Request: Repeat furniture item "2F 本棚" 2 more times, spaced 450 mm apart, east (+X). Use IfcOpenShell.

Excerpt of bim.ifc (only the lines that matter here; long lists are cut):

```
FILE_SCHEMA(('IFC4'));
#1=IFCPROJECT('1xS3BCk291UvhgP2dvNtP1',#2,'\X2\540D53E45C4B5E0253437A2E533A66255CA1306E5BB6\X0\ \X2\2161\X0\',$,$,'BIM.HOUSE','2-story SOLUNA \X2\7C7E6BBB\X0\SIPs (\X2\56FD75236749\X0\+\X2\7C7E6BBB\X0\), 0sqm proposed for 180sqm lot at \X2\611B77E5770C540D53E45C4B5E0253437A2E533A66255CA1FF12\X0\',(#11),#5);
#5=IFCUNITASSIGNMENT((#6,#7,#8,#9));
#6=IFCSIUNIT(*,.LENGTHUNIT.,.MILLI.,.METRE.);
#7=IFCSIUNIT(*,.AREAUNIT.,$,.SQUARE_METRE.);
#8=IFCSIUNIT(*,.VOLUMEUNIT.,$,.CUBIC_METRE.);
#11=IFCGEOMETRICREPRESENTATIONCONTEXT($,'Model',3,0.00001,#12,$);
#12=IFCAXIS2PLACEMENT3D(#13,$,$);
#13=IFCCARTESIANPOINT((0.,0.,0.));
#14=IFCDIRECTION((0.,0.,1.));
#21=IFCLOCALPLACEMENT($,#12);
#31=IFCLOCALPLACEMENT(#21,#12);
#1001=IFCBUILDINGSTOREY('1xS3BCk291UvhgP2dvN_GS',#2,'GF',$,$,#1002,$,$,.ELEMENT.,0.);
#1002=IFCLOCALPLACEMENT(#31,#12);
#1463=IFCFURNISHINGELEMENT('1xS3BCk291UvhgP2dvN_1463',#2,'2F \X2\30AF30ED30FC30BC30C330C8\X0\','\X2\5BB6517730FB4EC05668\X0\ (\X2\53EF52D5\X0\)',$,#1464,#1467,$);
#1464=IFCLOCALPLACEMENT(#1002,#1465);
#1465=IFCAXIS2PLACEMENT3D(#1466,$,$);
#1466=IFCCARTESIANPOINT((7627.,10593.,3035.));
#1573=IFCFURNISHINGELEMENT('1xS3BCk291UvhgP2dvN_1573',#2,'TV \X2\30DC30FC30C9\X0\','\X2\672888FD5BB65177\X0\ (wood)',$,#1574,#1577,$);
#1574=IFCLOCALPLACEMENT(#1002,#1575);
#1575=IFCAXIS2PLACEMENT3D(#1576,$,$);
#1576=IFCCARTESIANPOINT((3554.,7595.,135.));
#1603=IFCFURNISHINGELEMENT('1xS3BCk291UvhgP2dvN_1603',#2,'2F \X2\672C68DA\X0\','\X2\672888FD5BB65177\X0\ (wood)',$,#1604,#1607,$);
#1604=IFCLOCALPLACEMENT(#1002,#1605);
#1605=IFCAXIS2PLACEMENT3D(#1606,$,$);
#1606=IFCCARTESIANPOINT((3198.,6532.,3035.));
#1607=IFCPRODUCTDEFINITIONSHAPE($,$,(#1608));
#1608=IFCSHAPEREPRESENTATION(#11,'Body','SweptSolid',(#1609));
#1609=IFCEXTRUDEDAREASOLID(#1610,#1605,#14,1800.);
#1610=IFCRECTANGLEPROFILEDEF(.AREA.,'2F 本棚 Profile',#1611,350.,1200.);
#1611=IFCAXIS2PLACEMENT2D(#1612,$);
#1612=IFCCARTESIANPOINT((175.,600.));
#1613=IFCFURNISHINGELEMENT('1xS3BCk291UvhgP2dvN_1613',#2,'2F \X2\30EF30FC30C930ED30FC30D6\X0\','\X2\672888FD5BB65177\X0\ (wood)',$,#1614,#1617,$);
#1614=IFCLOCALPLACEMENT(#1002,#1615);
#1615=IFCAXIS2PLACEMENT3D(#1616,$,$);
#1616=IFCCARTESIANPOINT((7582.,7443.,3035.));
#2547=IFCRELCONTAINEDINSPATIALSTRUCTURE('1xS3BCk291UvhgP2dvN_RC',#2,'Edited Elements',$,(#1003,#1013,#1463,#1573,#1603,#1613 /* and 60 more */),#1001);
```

```python
import numpy as np
import ifcopenshell
import ifcopenshell.api.geometry
import ifcopenshell.api.root
import ifcopenshell.util.element
import ifcopenshell.util.placement

model = ifcopenshell.open("bim.ifc")


def reuse_history(source, copy):
    """copy_class also copies each property set's owner history, people and application; keep the originals."""
    for rel in copy.IsDefinedBy:
        if rel.is_a("IfcRelDefinesByProperties") and (history := rel.RelatingPropertyDefinition.OwnerHistory):
            rel.RelatingPropertyDefinition.OwnerHistory = source.OwnerHistory
            ifcopenshell.util.element.remove_deep2(model, history)


source = model.by_guid("1xS3BCk291UvhgP2dvN_1603")
base = ifcopenshell.util.placement.get_local_placement(source.ObjectPlacement)
step = np.array([1.0, 0.0, 0.0]) * 450.0

for i in range(1, 3):
    copy = ifcopenshell.api.root.copy_class(model, product=source)
    copy.Representation = ifcopenshell.util.element.copy_deep(
        model, source.Representation, exclude=["IfcGeometricRepresentationContext", "IfcRepresentationMap"]
    )
    reuse_history(source, copy)
    matrix = base.copy()
    matrix[:3, 3] += i * step
    print("added at", matrix[:3, 3].round(3) + 0.0)
    ifcopenshell.api.geometry.edit_object_placement(model, product=copy, matrix=matrix, is_si=False)

model.write("bim-out.ifc")
```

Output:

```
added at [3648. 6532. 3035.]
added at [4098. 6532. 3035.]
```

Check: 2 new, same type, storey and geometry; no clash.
